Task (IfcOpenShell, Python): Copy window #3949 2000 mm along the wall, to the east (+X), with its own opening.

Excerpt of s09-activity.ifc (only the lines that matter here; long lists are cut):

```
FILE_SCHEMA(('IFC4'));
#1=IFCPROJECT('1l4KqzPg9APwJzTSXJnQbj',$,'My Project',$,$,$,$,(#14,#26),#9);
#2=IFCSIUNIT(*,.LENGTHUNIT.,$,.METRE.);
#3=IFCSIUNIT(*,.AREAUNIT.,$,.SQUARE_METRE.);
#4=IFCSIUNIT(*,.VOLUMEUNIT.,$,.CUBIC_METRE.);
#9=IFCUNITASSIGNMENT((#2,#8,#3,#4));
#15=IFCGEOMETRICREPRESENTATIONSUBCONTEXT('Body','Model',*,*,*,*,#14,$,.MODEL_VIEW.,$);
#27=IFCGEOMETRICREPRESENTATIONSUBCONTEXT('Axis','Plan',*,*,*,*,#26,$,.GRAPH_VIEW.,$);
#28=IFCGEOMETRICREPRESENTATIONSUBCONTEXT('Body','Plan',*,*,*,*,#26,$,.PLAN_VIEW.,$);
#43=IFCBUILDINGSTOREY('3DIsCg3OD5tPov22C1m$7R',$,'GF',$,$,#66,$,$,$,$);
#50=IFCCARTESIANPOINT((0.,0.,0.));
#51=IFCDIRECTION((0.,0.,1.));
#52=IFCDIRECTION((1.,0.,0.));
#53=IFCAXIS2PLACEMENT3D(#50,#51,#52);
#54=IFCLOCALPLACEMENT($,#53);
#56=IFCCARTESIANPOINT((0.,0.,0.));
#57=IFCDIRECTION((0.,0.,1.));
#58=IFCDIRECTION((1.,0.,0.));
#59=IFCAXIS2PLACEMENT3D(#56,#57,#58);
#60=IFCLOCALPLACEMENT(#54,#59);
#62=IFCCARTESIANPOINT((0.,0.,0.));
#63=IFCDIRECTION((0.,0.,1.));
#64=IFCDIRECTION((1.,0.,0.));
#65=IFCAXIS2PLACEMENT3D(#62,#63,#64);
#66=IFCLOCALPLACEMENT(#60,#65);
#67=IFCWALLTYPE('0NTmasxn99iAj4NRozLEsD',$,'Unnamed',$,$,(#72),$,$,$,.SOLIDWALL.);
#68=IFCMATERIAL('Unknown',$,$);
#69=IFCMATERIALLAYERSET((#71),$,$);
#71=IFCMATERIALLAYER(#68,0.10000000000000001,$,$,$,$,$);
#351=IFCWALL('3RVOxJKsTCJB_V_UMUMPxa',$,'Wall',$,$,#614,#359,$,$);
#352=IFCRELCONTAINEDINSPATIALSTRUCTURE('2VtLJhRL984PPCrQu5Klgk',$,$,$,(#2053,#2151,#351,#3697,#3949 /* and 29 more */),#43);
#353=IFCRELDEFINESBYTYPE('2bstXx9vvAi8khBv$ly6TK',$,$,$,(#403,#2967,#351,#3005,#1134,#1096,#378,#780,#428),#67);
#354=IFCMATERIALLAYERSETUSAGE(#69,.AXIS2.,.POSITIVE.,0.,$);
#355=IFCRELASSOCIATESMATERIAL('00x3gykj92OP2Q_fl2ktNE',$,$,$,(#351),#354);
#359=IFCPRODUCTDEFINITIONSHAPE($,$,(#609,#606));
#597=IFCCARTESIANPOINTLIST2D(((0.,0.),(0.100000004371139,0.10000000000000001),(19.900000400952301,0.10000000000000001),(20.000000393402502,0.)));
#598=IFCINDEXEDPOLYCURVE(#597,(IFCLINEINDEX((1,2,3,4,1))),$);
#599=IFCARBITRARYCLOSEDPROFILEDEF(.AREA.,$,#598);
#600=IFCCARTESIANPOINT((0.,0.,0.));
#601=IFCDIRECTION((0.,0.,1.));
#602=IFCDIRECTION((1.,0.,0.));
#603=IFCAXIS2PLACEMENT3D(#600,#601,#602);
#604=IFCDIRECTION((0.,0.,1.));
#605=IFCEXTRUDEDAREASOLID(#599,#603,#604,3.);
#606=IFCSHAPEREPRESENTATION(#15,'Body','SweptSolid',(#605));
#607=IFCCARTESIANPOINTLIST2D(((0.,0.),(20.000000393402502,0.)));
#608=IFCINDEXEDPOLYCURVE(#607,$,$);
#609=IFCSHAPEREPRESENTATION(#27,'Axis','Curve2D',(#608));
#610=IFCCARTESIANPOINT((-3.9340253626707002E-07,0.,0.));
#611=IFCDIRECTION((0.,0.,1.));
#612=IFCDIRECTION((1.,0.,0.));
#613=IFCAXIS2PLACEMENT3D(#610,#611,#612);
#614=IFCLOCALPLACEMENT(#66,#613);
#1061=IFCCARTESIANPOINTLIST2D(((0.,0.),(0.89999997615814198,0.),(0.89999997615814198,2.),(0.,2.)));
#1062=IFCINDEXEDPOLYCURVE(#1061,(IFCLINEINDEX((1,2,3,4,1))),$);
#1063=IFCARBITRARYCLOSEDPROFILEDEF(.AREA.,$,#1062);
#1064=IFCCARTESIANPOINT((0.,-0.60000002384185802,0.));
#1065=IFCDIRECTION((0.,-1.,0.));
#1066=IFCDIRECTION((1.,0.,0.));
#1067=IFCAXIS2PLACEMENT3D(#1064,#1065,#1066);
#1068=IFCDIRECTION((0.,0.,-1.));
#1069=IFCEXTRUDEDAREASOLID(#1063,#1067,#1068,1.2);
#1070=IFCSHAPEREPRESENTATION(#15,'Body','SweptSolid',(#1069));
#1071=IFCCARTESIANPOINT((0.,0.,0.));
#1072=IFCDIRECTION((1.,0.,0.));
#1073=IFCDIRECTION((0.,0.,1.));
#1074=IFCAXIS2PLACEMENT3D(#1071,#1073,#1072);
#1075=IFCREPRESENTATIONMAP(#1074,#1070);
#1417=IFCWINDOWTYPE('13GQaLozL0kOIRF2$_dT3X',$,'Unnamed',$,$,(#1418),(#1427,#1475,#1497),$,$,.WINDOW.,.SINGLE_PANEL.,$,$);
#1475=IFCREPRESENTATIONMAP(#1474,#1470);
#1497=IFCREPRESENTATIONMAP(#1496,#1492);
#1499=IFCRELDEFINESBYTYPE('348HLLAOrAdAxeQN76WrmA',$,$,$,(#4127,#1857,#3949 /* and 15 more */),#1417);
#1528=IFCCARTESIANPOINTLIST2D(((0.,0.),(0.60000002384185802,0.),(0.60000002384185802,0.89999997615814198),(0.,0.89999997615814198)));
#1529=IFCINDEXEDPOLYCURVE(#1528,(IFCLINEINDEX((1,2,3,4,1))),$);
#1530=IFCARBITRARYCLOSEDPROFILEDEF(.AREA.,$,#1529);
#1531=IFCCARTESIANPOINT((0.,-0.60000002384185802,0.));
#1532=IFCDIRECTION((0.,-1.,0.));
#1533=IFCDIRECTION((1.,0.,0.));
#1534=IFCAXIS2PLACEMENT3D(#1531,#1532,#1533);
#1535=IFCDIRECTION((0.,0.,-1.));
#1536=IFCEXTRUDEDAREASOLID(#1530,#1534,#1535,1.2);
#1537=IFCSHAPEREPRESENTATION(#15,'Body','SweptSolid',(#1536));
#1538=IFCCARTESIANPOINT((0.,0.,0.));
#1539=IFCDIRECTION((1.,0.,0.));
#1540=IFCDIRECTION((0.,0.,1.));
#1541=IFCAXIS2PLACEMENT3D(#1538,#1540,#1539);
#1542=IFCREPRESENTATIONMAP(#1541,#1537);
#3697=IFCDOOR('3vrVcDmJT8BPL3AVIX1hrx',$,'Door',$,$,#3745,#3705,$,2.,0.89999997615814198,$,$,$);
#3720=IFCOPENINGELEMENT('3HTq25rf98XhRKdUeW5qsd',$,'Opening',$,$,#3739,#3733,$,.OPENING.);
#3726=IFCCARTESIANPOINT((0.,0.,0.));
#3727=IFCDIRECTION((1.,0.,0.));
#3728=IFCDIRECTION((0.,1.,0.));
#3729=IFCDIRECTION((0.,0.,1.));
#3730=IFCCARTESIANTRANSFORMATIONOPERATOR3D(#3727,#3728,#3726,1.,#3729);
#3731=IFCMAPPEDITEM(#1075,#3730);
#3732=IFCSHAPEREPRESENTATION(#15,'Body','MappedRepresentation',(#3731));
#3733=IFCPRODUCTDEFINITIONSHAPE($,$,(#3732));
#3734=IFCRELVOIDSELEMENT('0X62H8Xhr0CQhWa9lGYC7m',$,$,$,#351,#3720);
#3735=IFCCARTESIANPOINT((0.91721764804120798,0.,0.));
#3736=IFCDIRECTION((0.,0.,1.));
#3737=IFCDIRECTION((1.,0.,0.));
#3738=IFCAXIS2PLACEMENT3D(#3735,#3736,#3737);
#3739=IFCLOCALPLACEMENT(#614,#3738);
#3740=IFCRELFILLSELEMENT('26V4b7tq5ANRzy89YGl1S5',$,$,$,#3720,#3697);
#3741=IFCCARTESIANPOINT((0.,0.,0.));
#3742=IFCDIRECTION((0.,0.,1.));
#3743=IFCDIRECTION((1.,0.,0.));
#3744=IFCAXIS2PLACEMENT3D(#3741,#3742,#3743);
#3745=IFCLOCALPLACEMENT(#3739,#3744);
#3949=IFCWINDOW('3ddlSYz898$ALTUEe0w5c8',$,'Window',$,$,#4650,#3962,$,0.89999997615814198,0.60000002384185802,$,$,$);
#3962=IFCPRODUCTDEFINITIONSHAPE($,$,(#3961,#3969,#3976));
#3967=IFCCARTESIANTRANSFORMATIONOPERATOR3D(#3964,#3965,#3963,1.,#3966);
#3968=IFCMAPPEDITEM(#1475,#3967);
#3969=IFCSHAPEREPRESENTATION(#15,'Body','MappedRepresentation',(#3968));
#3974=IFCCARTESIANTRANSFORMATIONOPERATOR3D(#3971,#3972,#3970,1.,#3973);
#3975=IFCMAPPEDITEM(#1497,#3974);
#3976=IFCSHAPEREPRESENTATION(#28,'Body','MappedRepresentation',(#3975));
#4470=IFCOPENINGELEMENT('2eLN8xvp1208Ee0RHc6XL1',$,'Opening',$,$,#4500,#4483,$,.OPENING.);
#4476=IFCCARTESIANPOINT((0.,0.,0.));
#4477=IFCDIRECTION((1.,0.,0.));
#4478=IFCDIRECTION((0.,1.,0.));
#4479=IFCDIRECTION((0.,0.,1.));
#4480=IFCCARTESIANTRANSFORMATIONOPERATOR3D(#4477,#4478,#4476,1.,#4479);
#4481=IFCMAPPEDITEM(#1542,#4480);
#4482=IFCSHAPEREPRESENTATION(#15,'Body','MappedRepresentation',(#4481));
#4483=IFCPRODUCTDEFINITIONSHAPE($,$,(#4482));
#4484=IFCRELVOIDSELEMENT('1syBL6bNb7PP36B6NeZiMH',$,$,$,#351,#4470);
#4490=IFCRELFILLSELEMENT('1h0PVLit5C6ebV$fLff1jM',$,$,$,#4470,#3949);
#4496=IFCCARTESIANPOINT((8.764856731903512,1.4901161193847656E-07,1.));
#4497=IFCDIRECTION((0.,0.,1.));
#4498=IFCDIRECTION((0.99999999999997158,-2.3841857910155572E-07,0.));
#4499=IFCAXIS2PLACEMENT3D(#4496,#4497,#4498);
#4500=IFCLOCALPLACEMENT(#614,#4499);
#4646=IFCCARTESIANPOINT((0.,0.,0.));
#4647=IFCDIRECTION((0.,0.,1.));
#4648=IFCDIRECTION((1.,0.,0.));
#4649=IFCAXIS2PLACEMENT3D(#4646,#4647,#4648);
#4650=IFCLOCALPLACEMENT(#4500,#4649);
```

```python
import ifcopenshell
import ifcopenshell.api.feature
import ifcopenshell.api.geometry
import ifcopenshell.api.root
import ifcopenshell.geom
import ifcopenshell.util.element
import ifcopenshell.util.placement
import ifcopenshell.util.shape

model = ifcopenshell.open("s09-activity.ifc")
settings = ifcopenshell.geom.settings()


def volume(element):
    """Net volume in cubic metres, openings subtracted."""
    shape = ifcopenshell.geom.create_shape(settings, element)
    return ifcopenshell.util.shape.get_volume(shape.geometry)


window = model.by_guid("3ddlSYz898$ALTUEe0w5c8")
opening = window.FillsVoids[0].RelatingOpeningElement
wall = opening.VoidsElements[0].RelatingBuildingElement
before = volume(wall)
shift = ifcopenshell.util.placement.get_local_placement(wall.ObjectPlacement)[:3, 0] * 2.0

# copy_class copies the void relationship, type, container and properties, but no geometry.
new_opening = ifcopenshell.api.root.copy_class(model, product=opening)
new_opening.Representation = ifcopenshell.util.element.copy_deep(
    model, opening.Representation, exclude=["IfcGeometricRepresentationContext", "IfcRepresentationMap"]
)
new_window = ifcopenshell.api.root.copy_class(model, product=window)
new_window.Representation = ifcopenshell.util.element.copy_deep(
    model, window.Representation, exclude=["IfcGeometricRepresentationContext", "IfcRepresentationMap"]
)
ifcopenshell.api.feature.add_filling(model, opening=new_opening, element=new_window)

for old, new in ((opening, new_opening), (window, new_window)):
    matrix = ifcopenshell.util.placement.get_local_placement(old.ObjectPlacement)
    matrix[:3, 3] += shift
    ifcopenshell.api.geometry.edit_object_placement(model, product=new, matrix=matrix, is_si=False)

after = volume(wall)

print(f"wall volume {before:.3f} -> {after:.3f} m3")

model.write("s09-activity-out.ifc")
```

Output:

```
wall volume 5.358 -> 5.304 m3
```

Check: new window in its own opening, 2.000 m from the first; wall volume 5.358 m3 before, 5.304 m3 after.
